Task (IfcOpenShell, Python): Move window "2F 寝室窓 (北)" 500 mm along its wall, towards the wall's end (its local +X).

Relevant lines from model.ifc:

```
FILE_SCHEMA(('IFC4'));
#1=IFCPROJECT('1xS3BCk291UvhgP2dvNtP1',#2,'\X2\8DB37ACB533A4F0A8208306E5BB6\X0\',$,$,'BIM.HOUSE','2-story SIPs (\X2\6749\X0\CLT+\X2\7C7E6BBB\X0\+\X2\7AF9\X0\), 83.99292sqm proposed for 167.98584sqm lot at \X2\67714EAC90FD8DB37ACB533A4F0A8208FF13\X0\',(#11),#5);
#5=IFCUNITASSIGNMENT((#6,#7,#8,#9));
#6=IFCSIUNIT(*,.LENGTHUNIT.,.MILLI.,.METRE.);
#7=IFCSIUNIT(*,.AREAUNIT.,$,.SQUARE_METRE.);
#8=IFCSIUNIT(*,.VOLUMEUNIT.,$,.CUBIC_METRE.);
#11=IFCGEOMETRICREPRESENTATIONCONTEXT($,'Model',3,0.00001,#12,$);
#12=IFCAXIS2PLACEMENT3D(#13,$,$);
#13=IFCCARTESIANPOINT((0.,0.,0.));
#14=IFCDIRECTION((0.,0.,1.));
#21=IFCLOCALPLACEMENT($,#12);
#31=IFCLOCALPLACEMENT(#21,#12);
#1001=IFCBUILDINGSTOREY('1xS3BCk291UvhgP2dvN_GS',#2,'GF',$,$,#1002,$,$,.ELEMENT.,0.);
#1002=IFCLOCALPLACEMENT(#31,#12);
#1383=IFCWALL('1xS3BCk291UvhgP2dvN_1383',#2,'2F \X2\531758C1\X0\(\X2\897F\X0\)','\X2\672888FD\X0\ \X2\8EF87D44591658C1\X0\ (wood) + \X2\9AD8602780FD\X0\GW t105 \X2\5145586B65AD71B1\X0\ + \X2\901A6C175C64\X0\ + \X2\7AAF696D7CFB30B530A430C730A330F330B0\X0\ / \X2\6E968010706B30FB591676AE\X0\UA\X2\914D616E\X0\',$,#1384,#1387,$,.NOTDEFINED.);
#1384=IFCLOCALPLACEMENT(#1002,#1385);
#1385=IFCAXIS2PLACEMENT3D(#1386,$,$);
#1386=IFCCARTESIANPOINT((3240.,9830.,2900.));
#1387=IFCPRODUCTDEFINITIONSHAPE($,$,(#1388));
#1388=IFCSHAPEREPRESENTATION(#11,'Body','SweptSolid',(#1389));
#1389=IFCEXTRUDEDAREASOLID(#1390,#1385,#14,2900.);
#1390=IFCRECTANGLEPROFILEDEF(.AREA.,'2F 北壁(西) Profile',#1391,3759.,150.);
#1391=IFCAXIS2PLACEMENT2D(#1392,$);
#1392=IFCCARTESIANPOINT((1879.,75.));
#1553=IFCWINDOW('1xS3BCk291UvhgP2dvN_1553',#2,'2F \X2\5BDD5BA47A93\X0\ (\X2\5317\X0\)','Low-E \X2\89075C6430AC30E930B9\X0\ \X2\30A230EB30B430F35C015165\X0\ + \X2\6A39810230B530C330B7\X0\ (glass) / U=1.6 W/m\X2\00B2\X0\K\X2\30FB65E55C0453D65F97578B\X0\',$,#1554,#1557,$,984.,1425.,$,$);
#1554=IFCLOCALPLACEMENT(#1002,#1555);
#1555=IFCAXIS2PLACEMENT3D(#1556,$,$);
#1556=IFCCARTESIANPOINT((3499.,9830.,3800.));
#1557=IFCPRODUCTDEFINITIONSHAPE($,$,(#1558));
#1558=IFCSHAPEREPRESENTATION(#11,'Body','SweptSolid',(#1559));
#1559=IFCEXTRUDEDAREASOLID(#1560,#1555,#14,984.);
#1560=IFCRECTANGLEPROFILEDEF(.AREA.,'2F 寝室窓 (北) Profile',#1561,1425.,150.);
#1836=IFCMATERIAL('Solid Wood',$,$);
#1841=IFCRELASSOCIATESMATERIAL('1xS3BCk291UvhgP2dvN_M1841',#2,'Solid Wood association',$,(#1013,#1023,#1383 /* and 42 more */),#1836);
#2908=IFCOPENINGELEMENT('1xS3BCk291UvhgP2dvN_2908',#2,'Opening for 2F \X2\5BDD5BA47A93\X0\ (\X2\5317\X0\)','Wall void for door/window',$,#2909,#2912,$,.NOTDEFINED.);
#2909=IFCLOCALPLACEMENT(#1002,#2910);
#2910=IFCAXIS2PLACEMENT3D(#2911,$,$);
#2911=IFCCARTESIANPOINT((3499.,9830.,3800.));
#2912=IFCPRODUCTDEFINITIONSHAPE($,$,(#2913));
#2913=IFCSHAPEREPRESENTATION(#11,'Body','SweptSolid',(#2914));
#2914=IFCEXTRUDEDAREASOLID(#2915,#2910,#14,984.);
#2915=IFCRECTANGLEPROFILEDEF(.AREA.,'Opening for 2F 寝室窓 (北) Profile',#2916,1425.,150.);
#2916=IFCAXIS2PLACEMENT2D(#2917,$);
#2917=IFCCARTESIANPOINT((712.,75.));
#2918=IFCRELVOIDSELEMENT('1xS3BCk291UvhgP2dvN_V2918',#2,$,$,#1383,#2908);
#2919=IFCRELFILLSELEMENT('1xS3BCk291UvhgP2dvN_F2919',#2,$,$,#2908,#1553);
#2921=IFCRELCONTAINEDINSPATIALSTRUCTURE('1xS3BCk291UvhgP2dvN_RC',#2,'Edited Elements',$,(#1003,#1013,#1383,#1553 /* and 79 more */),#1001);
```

```python
import ifcopenshell
import ifcopenshell.api.geometry
import ifcopenshell.util.placement

model = ifcopenshell.open("model.ifc")

window = model.by_id(1553)
opening = window.FillsVoids[0].RelatingOpeningElement
wall = opening.VoidsElements[0].RelatingBuildingElement

wall_matrix = ifcopenshell.util.placement.get_local_placement(wall.ObjectPlacement)
shift = wall_matrix[:3, 0] * 500.0
before = ifcopenshell.util.placement.get_local_placement(window.ObjectPlacement)[:3, 3].copy()

# The window is not placed relative to its opening, so move both.
for product in (opening, window):
    matrix = ifcopenshell.util.placement.get_local_placement(product.ObjectPlacement)
    matrix[:3, 3] += shift
    ifcopenshell.api.geometry.edit_object_placement(model, product=product, matrix=matrix, is_si=False)

after = ifcopenshell.util.placement.get_local_placement(window.ObjectPlacement)[:3, 3]
print("window moved by", (after - before).round(3) + 0.0)

model.write("model_updated.ifc")
```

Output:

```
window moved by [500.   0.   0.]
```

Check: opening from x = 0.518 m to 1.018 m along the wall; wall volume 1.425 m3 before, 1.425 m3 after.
